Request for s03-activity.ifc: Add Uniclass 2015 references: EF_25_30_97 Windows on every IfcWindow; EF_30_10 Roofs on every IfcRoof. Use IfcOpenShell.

First a look at what the model holds.

```python
import ifcopenshell

model = ifcopenshell.open("s03-activity.ifc")
print(model.schema)
print("classifications:", [c.Name for c in model.by_type("IfcClassification")])
for ifc_class in ("IfcDoor", "IfcRoof", "IfcStair", "IfcWall", "IfcWindow"):
    print(ifc_class, len(model.by_type(ifc_class)))
```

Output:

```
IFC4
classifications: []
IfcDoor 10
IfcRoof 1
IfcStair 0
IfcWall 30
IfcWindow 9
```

```python
import ifcopenshell
import ifcopenshell.api.classification

model = ifcopenshell.open("s03-activity.ifc")

system = ifcopenshell.api.classification.add_classification(model, classification="Uniclass 2015")

codes = {
    "IfcWindow": ("EF_25_30_97", "Windows"),
    "IfcRoof": ("EF_30_10", "Roofs"),
}
for ifc_class, (code, name) in codes.items():
    products = model.by_type(ifc_class)
    ifcopenshell.api.classification.add_reference(
        model, products=products, classification=system, identification=code, name=name
    )
    print(code, len(products))

model.write("s03-activity_updated.ifc")
```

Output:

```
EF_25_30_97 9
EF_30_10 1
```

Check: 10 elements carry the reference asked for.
